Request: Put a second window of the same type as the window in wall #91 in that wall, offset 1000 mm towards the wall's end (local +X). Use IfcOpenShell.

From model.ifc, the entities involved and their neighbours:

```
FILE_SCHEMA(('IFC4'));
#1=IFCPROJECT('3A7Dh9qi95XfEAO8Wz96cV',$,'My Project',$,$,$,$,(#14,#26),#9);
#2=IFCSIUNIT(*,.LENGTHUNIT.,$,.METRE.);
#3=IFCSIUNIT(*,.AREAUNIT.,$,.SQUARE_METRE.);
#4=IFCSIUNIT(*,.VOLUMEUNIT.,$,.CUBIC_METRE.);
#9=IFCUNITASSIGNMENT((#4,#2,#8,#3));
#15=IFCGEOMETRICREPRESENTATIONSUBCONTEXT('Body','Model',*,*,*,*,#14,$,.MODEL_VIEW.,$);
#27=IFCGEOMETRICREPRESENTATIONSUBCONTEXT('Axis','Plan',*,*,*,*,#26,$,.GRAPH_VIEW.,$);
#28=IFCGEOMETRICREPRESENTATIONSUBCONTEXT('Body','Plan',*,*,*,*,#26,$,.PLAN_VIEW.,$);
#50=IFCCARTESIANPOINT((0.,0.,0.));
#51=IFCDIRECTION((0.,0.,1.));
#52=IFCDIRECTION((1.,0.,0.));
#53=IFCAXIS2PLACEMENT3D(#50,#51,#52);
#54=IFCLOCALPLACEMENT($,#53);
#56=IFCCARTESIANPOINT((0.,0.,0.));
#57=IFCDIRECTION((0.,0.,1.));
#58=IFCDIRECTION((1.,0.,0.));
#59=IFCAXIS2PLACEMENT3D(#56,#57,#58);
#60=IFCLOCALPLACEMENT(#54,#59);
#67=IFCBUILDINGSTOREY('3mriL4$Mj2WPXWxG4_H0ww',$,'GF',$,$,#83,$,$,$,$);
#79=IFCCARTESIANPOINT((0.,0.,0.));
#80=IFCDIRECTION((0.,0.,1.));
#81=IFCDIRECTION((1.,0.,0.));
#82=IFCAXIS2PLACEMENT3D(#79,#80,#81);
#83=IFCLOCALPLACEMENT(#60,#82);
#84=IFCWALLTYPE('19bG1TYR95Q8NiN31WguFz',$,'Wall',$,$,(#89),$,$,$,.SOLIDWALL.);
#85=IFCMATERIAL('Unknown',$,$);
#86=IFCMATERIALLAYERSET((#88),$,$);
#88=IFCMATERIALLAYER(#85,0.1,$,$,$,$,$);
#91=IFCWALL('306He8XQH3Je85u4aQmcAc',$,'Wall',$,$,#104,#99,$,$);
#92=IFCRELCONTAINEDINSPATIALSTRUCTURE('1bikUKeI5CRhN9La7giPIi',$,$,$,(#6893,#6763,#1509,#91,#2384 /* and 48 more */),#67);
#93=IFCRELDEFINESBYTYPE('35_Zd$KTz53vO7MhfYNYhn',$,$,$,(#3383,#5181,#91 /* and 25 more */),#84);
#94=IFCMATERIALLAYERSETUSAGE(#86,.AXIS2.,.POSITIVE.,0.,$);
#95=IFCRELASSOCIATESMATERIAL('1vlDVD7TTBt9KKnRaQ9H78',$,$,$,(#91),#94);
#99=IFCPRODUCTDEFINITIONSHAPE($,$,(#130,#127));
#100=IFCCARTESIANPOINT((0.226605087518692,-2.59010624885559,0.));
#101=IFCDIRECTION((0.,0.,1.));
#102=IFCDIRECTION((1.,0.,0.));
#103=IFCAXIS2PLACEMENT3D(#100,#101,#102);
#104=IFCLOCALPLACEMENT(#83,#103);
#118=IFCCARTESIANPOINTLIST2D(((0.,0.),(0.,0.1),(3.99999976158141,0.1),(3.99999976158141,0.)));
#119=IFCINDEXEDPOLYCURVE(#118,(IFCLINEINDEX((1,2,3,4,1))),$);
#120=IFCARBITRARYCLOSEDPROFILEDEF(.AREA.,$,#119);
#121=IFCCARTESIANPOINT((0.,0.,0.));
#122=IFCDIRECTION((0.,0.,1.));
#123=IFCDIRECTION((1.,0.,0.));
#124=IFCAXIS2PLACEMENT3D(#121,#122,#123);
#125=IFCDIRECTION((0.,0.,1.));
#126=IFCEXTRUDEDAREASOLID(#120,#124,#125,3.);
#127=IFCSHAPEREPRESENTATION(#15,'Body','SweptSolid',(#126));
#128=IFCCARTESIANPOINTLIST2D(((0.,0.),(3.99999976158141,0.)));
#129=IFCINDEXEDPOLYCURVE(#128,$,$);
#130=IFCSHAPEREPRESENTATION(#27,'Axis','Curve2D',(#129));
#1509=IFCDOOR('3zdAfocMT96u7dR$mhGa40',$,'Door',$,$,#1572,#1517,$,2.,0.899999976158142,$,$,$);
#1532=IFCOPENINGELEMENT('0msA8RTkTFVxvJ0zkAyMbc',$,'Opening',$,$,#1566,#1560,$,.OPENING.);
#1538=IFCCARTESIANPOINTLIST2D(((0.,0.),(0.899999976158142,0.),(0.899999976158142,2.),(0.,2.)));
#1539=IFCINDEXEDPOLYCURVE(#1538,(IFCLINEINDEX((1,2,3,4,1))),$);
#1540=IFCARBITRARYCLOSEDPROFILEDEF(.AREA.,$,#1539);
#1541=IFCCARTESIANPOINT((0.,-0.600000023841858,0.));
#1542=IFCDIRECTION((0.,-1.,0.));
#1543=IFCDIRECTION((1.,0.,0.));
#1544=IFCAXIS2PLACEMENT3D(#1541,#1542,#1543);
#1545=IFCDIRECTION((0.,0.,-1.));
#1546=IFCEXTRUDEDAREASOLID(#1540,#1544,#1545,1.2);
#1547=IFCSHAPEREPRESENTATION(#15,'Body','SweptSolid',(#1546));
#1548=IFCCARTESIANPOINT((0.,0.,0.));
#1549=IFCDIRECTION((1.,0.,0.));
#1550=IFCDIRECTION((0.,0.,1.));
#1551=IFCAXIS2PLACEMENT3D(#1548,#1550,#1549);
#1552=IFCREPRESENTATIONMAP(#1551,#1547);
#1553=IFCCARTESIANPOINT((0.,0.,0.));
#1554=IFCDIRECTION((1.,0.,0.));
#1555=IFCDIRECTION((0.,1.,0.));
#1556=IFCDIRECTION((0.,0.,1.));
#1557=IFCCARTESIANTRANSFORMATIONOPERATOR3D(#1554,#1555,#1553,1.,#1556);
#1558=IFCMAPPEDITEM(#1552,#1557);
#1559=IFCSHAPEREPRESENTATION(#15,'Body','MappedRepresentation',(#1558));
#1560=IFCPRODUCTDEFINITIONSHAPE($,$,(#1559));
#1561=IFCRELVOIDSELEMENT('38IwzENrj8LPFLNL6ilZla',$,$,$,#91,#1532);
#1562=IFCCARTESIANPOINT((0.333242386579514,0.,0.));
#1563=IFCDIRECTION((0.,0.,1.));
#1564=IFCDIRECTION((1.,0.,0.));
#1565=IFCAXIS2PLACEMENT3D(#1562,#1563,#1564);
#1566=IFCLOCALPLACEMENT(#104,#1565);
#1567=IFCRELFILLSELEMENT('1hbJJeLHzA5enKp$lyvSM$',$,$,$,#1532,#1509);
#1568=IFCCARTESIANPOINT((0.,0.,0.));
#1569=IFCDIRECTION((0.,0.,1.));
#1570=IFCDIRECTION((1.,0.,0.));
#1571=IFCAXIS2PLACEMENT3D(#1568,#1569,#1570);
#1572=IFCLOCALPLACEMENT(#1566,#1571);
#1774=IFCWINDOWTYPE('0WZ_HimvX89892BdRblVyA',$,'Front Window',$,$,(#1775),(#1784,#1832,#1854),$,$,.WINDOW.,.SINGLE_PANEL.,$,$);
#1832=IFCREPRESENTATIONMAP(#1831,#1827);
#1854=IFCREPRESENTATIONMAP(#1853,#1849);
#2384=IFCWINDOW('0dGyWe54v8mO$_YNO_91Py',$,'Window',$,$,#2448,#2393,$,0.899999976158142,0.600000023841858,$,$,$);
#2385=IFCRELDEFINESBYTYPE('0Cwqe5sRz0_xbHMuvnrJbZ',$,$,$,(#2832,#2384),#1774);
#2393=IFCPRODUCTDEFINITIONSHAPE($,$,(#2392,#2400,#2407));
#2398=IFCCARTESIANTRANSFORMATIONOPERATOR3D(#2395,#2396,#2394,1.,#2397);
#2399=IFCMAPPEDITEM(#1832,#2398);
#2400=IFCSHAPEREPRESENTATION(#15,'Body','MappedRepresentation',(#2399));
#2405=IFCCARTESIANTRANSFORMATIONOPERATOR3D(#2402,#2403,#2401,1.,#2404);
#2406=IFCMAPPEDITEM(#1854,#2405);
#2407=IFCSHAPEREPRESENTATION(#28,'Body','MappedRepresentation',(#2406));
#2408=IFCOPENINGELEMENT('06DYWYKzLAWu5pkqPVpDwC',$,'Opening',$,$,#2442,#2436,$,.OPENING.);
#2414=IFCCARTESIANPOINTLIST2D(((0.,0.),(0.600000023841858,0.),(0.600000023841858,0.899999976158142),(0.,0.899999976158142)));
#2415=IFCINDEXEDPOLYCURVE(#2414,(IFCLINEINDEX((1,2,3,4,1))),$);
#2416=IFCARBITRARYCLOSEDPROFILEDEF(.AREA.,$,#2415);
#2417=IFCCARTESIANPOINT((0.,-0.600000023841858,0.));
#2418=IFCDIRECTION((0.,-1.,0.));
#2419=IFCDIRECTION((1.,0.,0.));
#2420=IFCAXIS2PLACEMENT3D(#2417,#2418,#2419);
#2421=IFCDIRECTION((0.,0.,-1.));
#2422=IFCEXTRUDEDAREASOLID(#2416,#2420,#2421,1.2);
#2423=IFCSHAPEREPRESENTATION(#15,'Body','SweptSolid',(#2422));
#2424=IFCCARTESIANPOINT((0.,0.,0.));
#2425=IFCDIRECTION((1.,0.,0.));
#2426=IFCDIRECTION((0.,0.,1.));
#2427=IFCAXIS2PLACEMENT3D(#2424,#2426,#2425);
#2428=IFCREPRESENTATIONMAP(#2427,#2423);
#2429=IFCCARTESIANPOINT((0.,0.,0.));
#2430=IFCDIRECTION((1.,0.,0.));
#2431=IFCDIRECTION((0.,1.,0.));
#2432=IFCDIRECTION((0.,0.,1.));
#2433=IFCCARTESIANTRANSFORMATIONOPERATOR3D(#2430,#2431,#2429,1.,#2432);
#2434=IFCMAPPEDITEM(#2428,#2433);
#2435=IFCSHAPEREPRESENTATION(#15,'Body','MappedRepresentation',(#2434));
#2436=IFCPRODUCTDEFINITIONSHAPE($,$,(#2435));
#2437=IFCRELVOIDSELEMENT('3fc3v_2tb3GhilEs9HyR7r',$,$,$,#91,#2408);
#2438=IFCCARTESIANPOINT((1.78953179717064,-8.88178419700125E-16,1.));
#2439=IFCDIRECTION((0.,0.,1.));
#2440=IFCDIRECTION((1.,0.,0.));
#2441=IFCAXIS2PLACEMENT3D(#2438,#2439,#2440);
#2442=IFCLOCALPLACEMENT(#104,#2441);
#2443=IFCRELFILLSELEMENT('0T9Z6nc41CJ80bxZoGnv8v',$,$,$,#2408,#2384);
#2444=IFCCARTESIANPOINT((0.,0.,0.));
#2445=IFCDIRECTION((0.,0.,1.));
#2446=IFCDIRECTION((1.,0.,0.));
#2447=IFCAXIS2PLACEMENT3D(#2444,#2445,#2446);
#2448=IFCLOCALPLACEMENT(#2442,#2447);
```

```python
import ifcopenshell
import ifcopenshell.api.feature
import ifcopenshell.api.geometry
import ifcopenshell.api.root
import ifcopenshell.geom
import ifcopenshell.util.element
import ifcopenshell.util.placement
import ifcopenshell.util.shape
import ifcopenshell.util.unit

model = ifcopenshell.open("model.ifc")
unit_scale = ifcopenshell.util.unit.calculate_unit_scale(model)
settings = ifcopenshell.geom.settings()


def volume(element):
    """Net volume in cubic metres, openings subtracted."""
    shape = ifcopenshell.geom.create_shape(settings, element)
    return ifcopenshell.util.shape.get_volume(shape.geometry)


window = model.by_guid("0dGyWe54v8mO$_YNO_91Py")
opening = window.FillsVoids[0].RelatingOpeningElement
wall = opening.VoidsElements[0].RelatingBuildingElement
before = volume(wall)
shift = ifcopenshell.util.placement.get_local_placement(wall.ObjectPlacement)[:3, 0] * 1 / unit_scale

# copy_class copies the void relationship, type, container and properties, but no geometry.
new_opening = ifcopenshell.api.root.copy_class(model, product=opening)
new_opening.Representation = ifcopenshell.util.element.copy_deep(
    model, opening.Representation, exclude=["IfcGeometricRepresentationContext", "IfcRepresentationMap"]
)
new_window = ifcopenshell.api.root.copy_class(model, product=window)
new_window.Representation = ifcopenshell.util.element.copy_deep(
    model, window.Representation, exclude=["IfcGeometricRepresentationContext", "IfcRepresentationMap"]
)
ifcopenshell.api.feature.add_filling(model, opening=new_opening, element=new_window)

for old, new in ((opening, new_opening), (window, new_window)):
    matrix = ifcopenshell.util.placement.get_local_placement(old.ObjectPlacement)
    matrix[:3, 3] += shift
    ifcopenshell.api.geometry.edit_object_placement(model, product=new, matrix=matrix, is_si=False)

after = volume(wall)

print(f"wall volume {before:.3f} -> {after:.3f} m3")

model.write("model-out.ifc")
```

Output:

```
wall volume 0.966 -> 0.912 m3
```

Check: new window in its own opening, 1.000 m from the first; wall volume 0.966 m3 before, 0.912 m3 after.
